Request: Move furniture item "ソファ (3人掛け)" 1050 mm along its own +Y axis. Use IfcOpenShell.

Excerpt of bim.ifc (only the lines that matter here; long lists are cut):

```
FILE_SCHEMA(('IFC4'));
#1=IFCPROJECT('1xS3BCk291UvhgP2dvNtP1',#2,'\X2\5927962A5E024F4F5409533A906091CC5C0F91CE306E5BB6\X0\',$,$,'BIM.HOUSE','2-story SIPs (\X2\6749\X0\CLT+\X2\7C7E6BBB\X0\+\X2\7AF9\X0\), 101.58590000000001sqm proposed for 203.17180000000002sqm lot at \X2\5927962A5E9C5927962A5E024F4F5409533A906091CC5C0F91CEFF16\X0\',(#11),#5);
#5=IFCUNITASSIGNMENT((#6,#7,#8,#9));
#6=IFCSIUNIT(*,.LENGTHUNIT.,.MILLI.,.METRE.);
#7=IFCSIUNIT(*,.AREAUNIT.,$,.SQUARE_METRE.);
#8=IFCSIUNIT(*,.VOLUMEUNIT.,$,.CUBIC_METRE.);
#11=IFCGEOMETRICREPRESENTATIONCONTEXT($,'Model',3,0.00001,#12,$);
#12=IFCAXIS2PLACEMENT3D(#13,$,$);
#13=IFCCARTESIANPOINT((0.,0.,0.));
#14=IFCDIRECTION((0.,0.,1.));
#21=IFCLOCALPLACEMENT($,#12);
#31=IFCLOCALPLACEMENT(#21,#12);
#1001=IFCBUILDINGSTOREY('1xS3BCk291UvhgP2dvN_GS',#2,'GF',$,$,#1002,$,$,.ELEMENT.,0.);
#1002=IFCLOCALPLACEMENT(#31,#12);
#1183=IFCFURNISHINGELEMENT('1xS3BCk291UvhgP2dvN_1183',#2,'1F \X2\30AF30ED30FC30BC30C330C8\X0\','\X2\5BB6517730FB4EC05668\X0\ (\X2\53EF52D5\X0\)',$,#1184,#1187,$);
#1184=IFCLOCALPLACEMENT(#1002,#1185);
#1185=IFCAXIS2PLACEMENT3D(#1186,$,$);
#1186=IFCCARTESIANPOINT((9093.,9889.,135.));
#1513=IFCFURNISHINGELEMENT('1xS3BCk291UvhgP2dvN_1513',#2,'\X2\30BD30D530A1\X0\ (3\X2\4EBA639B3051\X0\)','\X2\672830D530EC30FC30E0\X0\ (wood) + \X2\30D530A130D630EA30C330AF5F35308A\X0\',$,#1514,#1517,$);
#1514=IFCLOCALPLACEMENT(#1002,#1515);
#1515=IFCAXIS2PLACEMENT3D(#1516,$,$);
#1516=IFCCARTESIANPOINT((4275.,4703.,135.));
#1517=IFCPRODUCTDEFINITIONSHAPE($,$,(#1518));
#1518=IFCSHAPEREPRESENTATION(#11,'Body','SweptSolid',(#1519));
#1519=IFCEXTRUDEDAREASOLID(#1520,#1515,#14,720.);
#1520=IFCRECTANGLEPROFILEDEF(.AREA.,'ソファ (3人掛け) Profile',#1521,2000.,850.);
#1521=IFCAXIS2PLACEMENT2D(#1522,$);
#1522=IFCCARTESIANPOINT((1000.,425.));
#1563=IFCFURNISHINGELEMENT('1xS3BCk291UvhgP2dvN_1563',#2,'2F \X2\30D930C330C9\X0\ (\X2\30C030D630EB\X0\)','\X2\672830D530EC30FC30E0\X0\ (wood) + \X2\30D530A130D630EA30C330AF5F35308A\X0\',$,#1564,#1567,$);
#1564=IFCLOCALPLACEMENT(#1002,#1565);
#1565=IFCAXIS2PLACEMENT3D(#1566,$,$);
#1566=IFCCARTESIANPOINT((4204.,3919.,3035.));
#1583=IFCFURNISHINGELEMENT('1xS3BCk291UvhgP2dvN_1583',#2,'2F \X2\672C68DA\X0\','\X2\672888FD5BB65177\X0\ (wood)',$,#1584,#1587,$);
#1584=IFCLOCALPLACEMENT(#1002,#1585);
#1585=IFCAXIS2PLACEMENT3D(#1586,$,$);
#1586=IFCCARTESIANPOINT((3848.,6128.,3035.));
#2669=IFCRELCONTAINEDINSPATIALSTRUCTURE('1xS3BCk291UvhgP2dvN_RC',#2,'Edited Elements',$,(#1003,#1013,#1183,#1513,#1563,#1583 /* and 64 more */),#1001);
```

```python
import ifcopenshell
import ifcopenshell.api.geometry
import ifcopenshell.util.placement
import ifcopenshell.util.unit

model = ifcopenshell.open("bim.ifc")
unit_scale = ifcopenshell.util.unit.calculate_unit_scale(model)

item = model.by_id(1513)
matrix = ifcopenshell.util.placement.get_local_placement(item.ObjectPlacement)
matrix[:3, 3] += matrix[:3, 1] * 1.05 / unit_scale
ifcopenshell.api.geometry.edit_object_placement(model, product=item, matrix=matrix, is_si=False)

print(ifcopenshell.util.placement.get_local_placement(item.ObjectPlacement).round(3) + 0.0)

model.write("bim_edited.ifc")
```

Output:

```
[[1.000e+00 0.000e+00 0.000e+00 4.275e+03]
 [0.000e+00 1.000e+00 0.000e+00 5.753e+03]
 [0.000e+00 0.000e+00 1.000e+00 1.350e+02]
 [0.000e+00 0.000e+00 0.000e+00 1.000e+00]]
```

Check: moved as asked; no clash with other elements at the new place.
